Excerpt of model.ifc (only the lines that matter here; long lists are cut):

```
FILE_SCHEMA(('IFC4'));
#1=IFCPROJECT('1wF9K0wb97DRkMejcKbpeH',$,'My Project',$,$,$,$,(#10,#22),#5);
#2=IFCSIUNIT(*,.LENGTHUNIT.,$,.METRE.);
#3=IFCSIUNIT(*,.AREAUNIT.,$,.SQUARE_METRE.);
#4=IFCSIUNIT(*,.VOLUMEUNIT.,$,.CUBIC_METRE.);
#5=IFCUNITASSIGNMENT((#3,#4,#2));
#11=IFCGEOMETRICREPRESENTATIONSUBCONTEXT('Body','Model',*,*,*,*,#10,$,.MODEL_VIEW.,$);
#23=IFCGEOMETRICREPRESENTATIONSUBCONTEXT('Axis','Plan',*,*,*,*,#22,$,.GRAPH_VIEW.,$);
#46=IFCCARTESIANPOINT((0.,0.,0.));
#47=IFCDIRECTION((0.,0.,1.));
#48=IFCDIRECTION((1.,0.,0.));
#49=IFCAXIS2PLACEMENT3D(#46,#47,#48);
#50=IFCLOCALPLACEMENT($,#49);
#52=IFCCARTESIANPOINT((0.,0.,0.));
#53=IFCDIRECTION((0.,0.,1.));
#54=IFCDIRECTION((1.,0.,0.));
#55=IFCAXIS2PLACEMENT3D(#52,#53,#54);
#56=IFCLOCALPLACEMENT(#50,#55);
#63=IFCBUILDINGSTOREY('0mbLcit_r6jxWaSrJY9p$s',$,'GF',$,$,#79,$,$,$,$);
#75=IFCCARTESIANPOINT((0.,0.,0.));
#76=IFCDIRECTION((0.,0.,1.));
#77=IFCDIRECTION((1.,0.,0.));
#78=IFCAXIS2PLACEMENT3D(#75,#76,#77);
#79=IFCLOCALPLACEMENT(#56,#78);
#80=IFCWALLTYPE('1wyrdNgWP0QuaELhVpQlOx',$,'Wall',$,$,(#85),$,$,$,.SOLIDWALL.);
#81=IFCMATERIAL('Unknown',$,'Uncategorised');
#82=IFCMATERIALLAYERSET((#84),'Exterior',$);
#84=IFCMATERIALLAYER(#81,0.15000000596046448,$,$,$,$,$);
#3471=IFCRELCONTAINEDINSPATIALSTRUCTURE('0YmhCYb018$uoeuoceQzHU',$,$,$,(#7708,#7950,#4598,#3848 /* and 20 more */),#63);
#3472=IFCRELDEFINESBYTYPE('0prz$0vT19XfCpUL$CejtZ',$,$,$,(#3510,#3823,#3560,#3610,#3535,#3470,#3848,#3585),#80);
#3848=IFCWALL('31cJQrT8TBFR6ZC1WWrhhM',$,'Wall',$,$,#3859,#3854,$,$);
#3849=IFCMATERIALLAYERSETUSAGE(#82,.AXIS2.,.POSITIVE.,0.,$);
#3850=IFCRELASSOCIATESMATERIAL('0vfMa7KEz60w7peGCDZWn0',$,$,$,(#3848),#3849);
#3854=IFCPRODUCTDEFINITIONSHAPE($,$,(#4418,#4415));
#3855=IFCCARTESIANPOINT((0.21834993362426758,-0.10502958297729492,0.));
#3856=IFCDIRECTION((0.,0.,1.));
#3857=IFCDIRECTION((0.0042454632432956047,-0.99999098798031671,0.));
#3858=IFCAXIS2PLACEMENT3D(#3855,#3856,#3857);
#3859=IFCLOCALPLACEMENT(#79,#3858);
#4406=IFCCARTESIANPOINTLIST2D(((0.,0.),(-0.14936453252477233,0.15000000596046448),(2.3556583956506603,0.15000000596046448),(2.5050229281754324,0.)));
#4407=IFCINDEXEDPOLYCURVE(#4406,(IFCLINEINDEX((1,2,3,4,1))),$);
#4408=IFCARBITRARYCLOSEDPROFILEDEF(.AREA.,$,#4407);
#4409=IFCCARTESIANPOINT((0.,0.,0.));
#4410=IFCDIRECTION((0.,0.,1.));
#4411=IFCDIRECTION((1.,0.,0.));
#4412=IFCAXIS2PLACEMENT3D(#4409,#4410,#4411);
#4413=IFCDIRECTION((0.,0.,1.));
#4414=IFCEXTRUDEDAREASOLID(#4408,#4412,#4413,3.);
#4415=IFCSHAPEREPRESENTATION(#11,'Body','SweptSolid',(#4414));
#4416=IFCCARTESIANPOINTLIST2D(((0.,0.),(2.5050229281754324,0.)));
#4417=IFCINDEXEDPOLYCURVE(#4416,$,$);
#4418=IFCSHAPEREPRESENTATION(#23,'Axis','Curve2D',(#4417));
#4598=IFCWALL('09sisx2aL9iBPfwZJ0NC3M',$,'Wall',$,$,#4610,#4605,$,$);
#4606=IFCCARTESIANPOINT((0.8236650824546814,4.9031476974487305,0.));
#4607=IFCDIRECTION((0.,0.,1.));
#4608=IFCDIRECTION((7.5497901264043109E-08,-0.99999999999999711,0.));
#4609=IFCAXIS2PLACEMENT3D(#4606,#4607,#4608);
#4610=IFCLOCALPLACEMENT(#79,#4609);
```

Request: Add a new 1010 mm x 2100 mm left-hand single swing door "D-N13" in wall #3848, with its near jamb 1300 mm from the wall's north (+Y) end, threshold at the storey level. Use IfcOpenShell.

```python
import numpy as np
import ifcopenshell
import ifcopenshell.api.feature
import ifcopenshell.api.geometry
import ifcopenshell.api.root
import ifcopenshell.api.spatial
import ifcopenshell.geom
import ifcopenshell.util.element
import ifcopenshell.util.placement
import ifcopenshell.util.representation
import ifcopenshell.util.shape
import ifcopenshell.util.unit

model = ifcopenshell.open("model.ifc")
unit_scale = ifcopenshell.util.unit.calculate_unit_scale(model)
settings = ifcopenshell.geom.settings()


def volume(element):
    """Net volume in cubic metres, openings subtracted."""
    shape = ifcopenshell.geom.create_shape(settings, element)
    return ifcopenshell.util.shape.get_volume(shape.geometry)


wall = model.by_guid("31cJQrT8TBFR6ZC1WWrhhM")
storey = ifcopenshell.util.element.get_container(wall, ifc_class="IfcBuildingStorey")
context = ifcopenshell.util.representation.get_context(model, "Model", "Body", "MODEL_VIEW")
before = volume(wall)

width, height, from_end, sill = 1.01, 2.1, 1.3, 0.0  # metres

# The wall runs along its own X axis, and the end named is its -X end.
wall_shape = ifcopenshell.geom.create_shape(settings, wall)
x, y, z = ifcopenshell.util.shape.get_vertices(wall_shape.geometry).T
start = x.min() + from_end
face, thickness = float(y.min()), float(y.max() - y.min())
wall_matrix = ifcopenshell.util.placement.get_local_placement(wall.ObjectPlacement)
level = ifcopenshell.util.placement.get_local_placement(storey.ObjectPlacement)[2, 3]


def in_wall(x, y):
    """Placement at x, y metres in the wall's axes, at sill height."""
    matrix = wall_matrix.copy()
    matrix[:, 3] = wall_matrix @ np.array([x / unit_scale, y / unit_scale, 0.0, 1.0])
    matrix[2, 3] = level + sill / unit_scale
    return matrix


# Opening: a box that overshoots both wall faces by 50 mm.
opening = ifcopenshell.api.root.create_entity(model, ifc_class="IfcOpeningElement", predefined_type="OPENING")
box = ifcopenshell.api.geometry.add_wall_representation(
    model, context=context, length=width, height=height, thickness=thickness + 0.1
)
ifcopenshell.api.geometry.assign_representation(model, product=opening, representation=box)
ifcopenshell.api.geometry.edit_object_placement(model, product=opening, matrix=in_wall(start, face - 0.05), is_si=False)
ifcopenshell.api.feature.add_feature(model, feature=opening, element=wall)

door = ifcopenshell.api.root.create_entity(model, ifc_class="IfcDoor", name="D-N13", predefined_type="DOOR")
door.OverallWidth, door.OverallHeight = width / unit_scale, height / unit_scale
door.OperationType = "SINGLE_SWING_LEFT"
body = ifcopenshell.api.geometry.add_door_representation(
    model,
    context=context,
    overall_width=door.OverallWidth,
    overall_height=door.OverallHeight,
    operation_type="SINGLE_SWING_LEFT",
    lining_properties={"LiningDepth": thickness / unit_scale, "ThresholdDepth": thickness / unit_scale},
)
ifcopenshell.api.geometry.assign_representation(model, product=door, representation=body)
ifcopenshell.api.spatial.assign_container(model, products=[door], relating_structure=storey)
ifcopenshell.api.feature.add_filling(model, opening=opening, element=door)

# The lining spans the wall, so the door starts at the wall face.
ifcopenshell.api.geometry.edit_object_placement(model, product=door, matrix=in_wall(start, face), is_si=False)

after = volume(wall)

print(f"wall volume {before:.3f} -> {after:.3f} m3")

model.write("model_edited.ifc")
```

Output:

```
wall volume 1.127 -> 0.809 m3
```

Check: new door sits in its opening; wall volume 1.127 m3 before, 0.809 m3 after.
